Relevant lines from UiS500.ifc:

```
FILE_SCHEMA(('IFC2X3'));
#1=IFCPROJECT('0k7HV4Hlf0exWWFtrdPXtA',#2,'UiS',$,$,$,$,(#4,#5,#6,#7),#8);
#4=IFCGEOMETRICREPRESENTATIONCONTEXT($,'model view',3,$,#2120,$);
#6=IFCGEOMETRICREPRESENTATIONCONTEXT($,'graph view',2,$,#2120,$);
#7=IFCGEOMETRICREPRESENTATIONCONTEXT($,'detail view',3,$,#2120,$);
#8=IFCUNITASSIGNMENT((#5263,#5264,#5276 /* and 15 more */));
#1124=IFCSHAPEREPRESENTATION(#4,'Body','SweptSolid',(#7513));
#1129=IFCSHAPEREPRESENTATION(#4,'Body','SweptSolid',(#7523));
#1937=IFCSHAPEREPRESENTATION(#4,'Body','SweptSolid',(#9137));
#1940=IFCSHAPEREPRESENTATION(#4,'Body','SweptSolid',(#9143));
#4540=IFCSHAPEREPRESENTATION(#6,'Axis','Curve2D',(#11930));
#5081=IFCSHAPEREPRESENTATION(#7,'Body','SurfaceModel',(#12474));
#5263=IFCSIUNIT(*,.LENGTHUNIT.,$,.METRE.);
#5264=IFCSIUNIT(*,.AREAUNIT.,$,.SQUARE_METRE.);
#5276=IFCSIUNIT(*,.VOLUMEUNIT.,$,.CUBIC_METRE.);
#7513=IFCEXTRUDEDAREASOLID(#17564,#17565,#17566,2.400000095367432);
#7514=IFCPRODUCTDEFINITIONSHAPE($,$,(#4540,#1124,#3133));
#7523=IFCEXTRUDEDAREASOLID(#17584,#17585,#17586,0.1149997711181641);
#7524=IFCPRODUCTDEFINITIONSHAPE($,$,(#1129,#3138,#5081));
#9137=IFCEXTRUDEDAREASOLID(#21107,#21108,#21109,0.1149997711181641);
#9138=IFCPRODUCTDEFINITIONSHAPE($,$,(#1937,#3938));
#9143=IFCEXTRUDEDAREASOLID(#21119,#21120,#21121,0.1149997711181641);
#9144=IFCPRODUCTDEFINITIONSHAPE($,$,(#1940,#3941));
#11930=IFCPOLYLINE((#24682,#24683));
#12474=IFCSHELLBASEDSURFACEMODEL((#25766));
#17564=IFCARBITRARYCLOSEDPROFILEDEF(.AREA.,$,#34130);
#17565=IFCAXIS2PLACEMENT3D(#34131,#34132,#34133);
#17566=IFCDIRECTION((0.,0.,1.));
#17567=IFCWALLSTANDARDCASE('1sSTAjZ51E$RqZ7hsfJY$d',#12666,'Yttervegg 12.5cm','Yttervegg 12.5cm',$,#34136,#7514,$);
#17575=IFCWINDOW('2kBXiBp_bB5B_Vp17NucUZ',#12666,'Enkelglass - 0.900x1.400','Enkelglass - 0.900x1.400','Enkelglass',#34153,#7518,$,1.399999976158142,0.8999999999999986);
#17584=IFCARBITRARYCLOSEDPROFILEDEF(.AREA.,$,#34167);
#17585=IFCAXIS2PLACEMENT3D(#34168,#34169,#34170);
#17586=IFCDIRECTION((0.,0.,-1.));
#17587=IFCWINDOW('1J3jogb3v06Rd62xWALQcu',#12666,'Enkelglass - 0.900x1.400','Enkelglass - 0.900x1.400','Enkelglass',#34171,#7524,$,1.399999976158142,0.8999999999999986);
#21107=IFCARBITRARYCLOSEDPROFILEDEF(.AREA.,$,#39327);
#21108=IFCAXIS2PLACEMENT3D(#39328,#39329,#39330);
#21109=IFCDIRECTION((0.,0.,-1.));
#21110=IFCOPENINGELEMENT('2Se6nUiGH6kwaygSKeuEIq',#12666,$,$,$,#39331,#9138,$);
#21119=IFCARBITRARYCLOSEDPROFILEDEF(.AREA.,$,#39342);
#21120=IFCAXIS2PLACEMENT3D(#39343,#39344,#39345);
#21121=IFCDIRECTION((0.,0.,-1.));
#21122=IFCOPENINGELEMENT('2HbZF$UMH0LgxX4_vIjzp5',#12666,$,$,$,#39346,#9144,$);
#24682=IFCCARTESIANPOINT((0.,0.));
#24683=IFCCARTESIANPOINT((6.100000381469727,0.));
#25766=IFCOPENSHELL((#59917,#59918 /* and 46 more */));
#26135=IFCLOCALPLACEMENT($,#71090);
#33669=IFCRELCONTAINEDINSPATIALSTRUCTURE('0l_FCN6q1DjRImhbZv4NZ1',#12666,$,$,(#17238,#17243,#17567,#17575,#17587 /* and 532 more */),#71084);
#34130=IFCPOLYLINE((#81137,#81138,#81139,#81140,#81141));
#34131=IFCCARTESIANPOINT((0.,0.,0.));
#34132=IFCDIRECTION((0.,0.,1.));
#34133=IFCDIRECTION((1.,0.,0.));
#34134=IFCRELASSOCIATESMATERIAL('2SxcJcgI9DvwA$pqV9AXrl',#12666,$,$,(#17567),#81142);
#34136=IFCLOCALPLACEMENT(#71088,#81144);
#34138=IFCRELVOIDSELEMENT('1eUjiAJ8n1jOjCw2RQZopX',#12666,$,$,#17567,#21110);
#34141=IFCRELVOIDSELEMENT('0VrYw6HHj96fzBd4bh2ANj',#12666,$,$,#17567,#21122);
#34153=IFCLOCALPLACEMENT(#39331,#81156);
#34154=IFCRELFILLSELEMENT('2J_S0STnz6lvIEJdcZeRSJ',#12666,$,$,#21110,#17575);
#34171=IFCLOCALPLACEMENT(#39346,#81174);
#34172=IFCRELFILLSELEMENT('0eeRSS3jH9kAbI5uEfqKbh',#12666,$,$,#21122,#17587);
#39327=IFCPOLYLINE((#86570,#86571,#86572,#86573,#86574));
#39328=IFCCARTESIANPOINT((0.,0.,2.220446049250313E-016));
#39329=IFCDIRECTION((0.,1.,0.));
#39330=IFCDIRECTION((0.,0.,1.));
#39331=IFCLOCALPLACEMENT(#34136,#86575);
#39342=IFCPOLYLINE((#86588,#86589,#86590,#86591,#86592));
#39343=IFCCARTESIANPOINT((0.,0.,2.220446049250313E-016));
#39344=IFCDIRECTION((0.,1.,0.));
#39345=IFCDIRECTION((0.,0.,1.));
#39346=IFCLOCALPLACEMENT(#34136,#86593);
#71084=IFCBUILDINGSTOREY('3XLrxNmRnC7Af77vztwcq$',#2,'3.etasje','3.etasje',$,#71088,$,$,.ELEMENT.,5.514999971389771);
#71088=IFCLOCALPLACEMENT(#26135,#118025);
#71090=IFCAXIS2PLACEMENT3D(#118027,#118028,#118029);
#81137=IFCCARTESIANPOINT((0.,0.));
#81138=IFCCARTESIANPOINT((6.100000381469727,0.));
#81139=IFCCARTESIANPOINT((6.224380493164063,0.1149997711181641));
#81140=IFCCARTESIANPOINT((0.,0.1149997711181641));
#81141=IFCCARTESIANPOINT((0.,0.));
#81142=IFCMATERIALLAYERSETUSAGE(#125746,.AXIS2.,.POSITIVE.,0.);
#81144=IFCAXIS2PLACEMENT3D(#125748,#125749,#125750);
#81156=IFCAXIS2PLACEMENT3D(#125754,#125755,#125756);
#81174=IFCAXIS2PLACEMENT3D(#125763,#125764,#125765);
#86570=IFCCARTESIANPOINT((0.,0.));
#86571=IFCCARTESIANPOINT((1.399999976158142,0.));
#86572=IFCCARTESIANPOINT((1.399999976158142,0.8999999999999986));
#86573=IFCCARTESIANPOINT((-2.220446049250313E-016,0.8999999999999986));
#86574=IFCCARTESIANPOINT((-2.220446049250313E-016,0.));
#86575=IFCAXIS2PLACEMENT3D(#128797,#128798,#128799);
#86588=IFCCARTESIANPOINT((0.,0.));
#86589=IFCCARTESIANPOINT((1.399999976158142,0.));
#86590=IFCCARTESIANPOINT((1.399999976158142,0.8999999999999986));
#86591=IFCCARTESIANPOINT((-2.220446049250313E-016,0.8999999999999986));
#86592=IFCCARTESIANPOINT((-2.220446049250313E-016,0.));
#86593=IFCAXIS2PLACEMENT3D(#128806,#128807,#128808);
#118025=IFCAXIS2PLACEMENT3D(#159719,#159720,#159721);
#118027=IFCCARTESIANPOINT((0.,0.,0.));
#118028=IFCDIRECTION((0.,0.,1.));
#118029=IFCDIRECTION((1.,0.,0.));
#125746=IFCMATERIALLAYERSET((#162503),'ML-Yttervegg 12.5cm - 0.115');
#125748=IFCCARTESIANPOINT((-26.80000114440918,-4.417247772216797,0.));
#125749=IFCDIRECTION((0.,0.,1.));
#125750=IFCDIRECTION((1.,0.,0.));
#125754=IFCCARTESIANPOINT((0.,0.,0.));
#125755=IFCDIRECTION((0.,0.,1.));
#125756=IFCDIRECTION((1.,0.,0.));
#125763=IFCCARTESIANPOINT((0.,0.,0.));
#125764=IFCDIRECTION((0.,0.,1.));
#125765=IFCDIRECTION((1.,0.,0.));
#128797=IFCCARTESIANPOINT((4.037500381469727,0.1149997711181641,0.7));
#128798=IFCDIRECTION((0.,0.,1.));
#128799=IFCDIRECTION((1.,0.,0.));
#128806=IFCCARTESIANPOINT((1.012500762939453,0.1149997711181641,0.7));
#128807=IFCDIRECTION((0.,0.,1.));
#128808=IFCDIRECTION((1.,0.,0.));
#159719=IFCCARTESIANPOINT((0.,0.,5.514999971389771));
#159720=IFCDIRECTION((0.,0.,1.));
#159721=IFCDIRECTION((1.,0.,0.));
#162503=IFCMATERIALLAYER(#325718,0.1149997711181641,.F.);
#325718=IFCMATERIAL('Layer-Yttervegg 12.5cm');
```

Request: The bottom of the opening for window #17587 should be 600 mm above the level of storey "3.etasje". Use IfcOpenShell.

```python
import numpy as np
import ifcopenshell
import ifcopenshell.api.geometry
import ifcopenshell.geom
import ifcopenshell.util.element
import ifcopenshell.util.placement
import ifcopenshell.util.shape
import ifcopenshell.util.unit

model = ifcopenshell.open("UiS500.ifc")
unit_scale = ifcopenshell.util.unit.calculate_unit_scale(model)

window = model.by_guid("1J3jogb3v06Rd62xWALQcu")
opening = window.FillsVoids[0].RelatingOpeningElement
storey = ifcopenshell.util.element.get_container(window, ifc_class="IfcBuildingStorey")
level = ifcopenshell.util.placement.get_local_placement(storey.ObjectPlacement)[2, 3]

# The opening's origin need not be at the sill, so measure its lowest point.
shape = ifcopenshell.geom.create_shape(ifcopenshell.geom.settings(), opening)
bottom = ifcopenshell.util.shape.get_shape_bottom_elevation(shape, shape.geometry) / unit_scale
dz = level + 0.6 / unit_scale - bottom

shift = np.array([0.0, 0.0, dz])
# The window is placed relative to its opening, so it follows when the opening moves.
matrix = ifcopenshell.util.placement.get_local_placement(opening.ObjectPlacement)
matrix[:3, 3] += shift
ifcopenshell.api.geometry.edit_object_placement(
    model, product=opening, matrix=matrix, is_si=False, should_transform_children=True
)

print(f"moved by {dz * unit_scale:+.3f} m")

model.write("UiS500-out.ifc")
```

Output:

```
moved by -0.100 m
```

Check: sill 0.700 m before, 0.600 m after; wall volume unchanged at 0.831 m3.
